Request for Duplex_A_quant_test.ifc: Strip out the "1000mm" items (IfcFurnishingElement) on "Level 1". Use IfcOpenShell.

First a look at what the model holds.

```python
import ifcopenshell
import ifcopenshell.util.element

model = ifcopenshell.open("Duplex_A_quant_test.ifc")
print(model.schema)
storey = next(s for s in model.by_type("IfcBuildingStorey") if s.Name == "Level 1")
furniture = [e for e in ifcopenshell.util.element.get_decomposition(storey) if e.is_a("IfcFurnishingElement")]
seen = {}
for e in furniture:
    element_type = ifcopenshell.util.element.get_type(e)
    name = element_type.Name if element_type not in (None, e) else None
    seen[name] = seen.get(name, 0) + 1
for name, count in sorted(seen.items(), key=str):
    print(count, "x", name)
```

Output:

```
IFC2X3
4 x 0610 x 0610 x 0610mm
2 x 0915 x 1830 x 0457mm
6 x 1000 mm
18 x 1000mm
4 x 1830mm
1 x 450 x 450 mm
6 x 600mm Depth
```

```python
import ifcopenshell
import ifcopenshell.api.root
import ifcopenshell.util.element

model = ifcopenshell.open("Duplex_A_quant_test.ifc")

storey = next(s for s in model.by_type("IfcBuildingStorey") if s.Name == "Level 1")
furniture = [e for e in ifcopenshell.util.element.get_decomposition(storey) if e.is_a("IfcFurnishingElement")]
targets = [e for e in furniture if (t := ifcopenshell.util.element.get_type(e)) not in (None, e) and t.Name == "1000mm"]

for e in targets:
    ifcopenshell.api.root.remove_product(model, product=e)
print(len(targets), "removed")

model.write("Duplex_A_quant_test-out.ifc")
```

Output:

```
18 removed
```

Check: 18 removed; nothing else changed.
